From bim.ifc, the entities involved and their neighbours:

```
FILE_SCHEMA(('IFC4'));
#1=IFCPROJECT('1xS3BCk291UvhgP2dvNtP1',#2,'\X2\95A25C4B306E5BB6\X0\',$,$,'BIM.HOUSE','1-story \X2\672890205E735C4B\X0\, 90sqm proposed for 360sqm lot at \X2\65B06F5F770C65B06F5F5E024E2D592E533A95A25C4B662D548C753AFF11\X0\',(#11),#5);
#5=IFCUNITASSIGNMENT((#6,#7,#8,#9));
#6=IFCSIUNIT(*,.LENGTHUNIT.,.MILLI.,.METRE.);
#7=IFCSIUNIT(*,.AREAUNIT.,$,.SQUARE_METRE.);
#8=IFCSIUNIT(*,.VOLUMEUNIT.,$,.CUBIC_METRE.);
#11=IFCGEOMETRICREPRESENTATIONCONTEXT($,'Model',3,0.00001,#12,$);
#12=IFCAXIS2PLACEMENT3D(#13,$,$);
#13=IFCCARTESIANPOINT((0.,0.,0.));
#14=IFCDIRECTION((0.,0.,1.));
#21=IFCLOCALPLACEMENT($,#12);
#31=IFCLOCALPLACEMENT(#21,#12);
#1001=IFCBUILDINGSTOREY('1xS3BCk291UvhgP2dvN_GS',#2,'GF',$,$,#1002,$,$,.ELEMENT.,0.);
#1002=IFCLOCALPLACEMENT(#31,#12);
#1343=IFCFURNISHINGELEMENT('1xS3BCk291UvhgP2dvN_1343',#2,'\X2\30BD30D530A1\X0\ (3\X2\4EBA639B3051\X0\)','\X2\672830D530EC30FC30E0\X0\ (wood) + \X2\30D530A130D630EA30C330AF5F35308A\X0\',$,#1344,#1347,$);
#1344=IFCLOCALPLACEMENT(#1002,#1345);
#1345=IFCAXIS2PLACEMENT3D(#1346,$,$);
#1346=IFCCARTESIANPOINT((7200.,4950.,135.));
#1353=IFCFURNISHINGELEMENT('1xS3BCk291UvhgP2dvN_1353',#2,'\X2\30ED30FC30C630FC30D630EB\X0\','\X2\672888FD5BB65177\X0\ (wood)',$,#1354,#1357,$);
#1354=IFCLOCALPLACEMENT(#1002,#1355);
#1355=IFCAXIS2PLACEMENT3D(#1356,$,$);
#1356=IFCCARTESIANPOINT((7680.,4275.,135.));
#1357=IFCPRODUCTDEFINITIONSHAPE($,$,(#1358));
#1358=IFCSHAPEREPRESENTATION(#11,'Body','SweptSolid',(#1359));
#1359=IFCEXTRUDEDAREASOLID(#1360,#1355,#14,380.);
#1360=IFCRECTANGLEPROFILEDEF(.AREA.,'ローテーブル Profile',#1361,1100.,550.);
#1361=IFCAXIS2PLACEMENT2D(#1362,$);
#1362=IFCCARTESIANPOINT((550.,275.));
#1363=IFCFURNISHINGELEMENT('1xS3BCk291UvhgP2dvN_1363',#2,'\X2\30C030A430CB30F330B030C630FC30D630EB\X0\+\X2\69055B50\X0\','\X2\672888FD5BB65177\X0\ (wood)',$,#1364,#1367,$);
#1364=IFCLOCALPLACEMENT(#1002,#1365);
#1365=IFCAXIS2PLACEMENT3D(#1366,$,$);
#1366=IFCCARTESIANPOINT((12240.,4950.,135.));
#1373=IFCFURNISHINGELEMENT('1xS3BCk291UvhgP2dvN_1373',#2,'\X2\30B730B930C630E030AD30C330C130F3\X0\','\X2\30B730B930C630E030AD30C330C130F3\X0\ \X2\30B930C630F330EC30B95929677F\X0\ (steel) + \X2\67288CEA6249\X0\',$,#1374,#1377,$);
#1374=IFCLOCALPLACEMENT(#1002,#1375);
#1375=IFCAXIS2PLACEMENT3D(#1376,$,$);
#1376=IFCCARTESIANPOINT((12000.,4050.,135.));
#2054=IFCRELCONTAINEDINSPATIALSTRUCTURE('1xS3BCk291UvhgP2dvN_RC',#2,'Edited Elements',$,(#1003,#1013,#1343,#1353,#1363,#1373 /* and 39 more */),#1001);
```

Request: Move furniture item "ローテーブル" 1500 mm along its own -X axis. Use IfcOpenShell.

```python
import ifcopenshell
import ifcopenshell.api.geometry
import ifcopenshell.util.placement

model = ifcopenshell.open("bim.ifc")

item = model.by_guid("1xS3BCk291UvhgP2dvN_1353")
matrix = ifcopenshell.util.placement.get_local_placement(item.ObjectPlacement)
matrix[:3, 3] -= matrix[:3, 0] * 1500.0
ifcopenshell.api.geometry.edit_object_placement(model, product=item, matrix=matrix, is_si=False)

print(ifcopenshell.util.placement.get_local_placement(item.ObjectPlacement).round(3) + 0.0)

model.write("bim_rev.ifc")
```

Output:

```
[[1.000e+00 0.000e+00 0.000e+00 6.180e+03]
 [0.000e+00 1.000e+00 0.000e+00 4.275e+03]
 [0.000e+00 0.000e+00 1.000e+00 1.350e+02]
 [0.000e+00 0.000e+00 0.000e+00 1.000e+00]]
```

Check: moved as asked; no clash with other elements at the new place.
